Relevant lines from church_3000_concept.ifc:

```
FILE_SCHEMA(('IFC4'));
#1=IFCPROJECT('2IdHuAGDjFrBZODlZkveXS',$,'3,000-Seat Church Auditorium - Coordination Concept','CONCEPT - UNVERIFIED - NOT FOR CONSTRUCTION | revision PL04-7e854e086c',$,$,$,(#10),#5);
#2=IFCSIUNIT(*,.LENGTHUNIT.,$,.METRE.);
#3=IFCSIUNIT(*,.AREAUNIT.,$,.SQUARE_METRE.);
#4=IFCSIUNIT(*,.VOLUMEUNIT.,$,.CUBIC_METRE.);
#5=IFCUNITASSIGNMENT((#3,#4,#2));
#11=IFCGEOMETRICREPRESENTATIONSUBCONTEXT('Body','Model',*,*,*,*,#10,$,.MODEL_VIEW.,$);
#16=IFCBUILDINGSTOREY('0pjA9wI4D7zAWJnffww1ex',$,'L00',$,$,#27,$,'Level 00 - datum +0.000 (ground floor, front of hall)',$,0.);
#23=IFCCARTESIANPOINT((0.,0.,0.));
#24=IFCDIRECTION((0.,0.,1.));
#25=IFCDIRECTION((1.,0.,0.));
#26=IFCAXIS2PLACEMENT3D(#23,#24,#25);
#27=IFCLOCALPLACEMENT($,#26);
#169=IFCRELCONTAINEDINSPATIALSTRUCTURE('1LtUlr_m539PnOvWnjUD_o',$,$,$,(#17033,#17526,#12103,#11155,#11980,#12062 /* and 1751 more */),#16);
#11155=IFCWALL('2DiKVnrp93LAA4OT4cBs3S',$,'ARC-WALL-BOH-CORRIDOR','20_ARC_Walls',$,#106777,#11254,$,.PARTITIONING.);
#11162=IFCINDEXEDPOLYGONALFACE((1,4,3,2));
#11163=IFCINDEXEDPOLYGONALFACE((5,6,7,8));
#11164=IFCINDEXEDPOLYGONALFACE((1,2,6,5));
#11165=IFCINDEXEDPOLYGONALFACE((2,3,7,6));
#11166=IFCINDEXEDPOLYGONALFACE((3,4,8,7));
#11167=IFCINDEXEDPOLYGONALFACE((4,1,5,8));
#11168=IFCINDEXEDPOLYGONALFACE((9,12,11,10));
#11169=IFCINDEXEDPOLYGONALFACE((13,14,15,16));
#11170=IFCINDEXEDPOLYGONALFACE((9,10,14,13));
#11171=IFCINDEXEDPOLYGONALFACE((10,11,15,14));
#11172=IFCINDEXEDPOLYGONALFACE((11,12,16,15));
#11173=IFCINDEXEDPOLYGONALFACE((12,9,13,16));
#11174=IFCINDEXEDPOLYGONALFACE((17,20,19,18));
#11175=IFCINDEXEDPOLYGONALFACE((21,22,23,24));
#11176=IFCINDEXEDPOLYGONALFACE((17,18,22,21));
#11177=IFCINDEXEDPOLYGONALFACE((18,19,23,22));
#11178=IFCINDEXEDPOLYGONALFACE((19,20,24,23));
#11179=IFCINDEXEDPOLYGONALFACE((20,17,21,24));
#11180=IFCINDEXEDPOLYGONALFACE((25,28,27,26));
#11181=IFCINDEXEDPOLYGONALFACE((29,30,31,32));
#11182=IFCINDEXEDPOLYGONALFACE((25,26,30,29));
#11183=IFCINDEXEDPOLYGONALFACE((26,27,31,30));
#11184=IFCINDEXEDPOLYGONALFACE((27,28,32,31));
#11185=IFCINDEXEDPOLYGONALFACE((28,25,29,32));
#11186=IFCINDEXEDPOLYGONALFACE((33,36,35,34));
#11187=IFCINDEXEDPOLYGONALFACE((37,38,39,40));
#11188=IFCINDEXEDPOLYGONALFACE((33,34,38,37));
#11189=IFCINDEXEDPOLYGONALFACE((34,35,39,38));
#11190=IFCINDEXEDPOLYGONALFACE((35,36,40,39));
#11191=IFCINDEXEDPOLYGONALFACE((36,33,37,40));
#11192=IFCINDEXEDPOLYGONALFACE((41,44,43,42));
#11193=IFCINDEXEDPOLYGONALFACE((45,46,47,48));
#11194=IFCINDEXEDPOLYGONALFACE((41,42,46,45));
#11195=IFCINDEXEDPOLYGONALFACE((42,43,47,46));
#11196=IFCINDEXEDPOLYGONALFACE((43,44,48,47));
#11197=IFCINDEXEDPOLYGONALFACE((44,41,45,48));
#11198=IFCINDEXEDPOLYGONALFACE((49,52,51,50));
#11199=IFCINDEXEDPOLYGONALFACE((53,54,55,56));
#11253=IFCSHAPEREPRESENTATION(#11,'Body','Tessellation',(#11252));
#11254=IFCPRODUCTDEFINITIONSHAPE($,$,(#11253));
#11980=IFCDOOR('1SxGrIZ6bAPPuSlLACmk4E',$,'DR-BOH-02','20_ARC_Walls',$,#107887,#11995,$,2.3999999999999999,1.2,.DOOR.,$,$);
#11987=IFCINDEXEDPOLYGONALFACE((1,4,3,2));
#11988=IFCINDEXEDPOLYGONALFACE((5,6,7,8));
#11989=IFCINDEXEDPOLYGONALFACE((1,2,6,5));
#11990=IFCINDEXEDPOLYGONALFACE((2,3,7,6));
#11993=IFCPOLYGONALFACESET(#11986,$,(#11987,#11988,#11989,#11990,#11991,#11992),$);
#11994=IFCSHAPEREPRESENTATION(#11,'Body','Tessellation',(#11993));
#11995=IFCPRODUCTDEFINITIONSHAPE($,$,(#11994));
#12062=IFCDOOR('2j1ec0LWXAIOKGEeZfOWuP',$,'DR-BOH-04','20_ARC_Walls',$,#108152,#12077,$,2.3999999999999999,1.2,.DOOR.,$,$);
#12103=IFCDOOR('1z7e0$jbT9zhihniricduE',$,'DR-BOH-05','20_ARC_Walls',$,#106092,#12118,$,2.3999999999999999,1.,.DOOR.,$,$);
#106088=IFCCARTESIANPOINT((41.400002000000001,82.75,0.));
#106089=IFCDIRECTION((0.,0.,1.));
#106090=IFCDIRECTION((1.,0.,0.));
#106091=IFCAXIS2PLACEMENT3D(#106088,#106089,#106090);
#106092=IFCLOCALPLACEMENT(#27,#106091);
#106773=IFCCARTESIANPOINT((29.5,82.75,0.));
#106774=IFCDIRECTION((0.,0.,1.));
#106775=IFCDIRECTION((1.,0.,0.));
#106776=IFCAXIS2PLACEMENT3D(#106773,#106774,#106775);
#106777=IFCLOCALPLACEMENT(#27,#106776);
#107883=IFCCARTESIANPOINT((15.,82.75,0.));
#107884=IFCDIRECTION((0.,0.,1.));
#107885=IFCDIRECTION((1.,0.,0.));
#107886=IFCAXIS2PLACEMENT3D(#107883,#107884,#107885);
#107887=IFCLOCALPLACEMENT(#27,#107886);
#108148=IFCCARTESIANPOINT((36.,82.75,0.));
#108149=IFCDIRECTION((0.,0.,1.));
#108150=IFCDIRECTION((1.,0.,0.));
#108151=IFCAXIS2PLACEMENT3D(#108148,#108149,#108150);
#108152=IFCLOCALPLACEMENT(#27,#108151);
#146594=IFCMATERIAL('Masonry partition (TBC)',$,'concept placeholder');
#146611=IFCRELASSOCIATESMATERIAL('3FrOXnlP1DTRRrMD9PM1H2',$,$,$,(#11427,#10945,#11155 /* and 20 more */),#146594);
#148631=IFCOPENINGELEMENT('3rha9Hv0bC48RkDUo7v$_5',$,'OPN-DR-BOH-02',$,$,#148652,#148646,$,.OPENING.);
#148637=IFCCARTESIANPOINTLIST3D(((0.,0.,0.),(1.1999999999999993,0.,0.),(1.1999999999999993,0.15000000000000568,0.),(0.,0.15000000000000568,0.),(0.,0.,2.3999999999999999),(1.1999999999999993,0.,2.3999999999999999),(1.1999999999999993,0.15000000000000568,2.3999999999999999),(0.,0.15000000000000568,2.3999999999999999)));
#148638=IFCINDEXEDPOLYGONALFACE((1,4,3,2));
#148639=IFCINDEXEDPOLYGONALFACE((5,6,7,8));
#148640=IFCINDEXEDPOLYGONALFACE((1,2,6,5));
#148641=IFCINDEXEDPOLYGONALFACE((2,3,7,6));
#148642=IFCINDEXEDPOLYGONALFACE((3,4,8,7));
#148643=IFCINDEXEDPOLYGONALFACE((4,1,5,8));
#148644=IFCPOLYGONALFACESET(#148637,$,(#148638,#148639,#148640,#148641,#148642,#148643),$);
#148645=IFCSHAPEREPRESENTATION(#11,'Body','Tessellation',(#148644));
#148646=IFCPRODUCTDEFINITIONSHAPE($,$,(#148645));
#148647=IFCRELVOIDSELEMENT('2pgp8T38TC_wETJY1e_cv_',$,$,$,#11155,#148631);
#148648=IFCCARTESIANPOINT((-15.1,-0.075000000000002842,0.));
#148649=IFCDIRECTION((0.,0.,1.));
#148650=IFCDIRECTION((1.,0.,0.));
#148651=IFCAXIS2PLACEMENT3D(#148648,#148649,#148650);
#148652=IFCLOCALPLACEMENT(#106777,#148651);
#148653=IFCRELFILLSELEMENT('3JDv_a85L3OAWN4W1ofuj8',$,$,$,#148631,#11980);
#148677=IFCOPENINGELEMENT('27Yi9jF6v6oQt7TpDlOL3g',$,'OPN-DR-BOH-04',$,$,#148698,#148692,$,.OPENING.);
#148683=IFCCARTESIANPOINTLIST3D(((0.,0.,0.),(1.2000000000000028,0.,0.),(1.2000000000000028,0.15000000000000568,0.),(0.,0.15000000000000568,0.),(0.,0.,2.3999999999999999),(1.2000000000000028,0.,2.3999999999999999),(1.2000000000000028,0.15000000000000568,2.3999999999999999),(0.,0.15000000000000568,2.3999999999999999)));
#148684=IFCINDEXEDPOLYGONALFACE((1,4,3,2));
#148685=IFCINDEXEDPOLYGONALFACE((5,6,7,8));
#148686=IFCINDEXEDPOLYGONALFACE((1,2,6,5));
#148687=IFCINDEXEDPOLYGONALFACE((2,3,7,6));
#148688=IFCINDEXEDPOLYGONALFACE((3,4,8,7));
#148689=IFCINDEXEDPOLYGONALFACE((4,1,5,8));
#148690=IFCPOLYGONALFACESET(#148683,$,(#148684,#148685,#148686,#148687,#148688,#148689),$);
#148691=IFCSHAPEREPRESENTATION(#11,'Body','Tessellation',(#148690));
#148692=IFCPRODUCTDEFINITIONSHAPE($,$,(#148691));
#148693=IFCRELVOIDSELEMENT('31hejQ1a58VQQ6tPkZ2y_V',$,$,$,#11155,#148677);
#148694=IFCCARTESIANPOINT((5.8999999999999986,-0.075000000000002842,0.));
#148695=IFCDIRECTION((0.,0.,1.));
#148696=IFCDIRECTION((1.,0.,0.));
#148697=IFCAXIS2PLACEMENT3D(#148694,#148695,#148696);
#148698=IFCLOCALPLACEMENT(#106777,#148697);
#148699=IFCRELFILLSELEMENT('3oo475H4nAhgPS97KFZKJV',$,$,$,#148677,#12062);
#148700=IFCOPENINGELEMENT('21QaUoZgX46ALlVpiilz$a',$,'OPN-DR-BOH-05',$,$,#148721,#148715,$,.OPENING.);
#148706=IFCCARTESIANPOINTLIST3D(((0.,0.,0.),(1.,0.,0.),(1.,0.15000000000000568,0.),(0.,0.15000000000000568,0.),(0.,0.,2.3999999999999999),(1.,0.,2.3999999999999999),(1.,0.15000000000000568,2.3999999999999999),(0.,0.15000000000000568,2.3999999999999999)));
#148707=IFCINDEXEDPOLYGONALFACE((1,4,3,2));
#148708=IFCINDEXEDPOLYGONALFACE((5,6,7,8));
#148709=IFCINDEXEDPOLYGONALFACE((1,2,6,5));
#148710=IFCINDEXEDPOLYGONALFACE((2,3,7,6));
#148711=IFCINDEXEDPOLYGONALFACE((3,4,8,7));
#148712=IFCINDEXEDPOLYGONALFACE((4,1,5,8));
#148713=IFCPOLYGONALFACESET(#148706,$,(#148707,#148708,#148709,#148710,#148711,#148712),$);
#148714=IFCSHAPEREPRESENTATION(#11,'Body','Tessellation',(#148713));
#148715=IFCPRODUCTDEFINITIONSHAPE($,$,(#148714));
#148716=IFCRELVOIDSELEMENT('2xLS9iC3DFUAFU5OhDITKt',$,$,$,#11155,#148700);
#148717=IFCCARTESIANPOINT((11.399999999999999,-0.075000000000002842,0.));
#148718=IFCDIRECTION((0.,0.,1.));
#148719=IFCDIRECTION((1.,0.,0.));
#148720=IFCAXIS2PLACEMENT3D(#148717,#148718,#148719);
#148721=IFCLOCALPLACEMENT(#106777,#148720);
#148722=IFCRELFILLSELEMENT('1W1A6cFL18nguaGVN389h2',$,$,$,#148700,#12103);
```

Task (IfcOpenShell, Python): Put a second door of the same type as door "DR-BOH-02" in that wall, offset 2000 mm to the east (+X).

```python
import ifcopenshell
import ifcopenshell.api.feature
import ifcopenshell.api.geometry
import ifcopenshell.api.root
import ifcopenshell.geom
import ifcopenshell.util.element
import ifcopenshell.util.placement
import ifcopenshell.util.shape
import ifcopenshell.util.unit

model = ifcopenshell.open("church_3000_concept.ifc")
unit_scale = ifcopenshell.util.unit.calculate_unit_scale(model)
settings = ifcopenshell.geom.settings()


def volume(element):
    """Net volume in cubic metres, openings subtracted."""
    shape = ifcopenshell.geom.create_shape(settings, element)
    return ifcopenshell.util.shape.get_volume(shape.geometry)


door = model.by_guid("1SxGrIZ6bAPPuSlLACmk4E")
opening = door.FillsVoids[0].RelatingOpeningElement
wall = opening.VoidsElements[0].RelatingBuildingElement
before = volume(wall)
shift = ifcopenshell.util.placement.get_local_placement(wall.ObjectPlacement)[:3, 0] * 2 / unit_scale

# copy_class copies the void relationship, type, container and properties, but no geometry.
new_opening = ifcopenshell.api.root.copy_class(model, product=opening)
new_opening.Representation = ifcopenshell.util.element.copy_deep(
    model, opening.Representation, exclude=["IfcGeometricRepresentationContext", "IfcRepresentationMap"]
)
new_door = ifcopenshell.api.root.copy_class(model, product=door)
new_door.Representation = ifcopenshell.util.element.copy_deep(
    model, door.Representation, exclude=["IfcGeometricRepresentationContext", "IfcRepresentationMap"]
)
ifcopenshell.api.feature.add_filling(model, opening=new_opening, element=new_door)

for old, new in ((opening, new_opening), (door, new_door)):
    matrix = ifcopenshell.util.placement.get_local_placement(old.ObjectPlacement)
    matrix[:3, 3] += shift
    ifcopenshell.api.geometry.edit_object_placement(model, product=new, matrix=matrix, is_si=False)

after = volume(wall)

print(f"wall volume {before:.3f} -> {after:.3f} m3")

model.write("church_3000_concept-out.ifc")
```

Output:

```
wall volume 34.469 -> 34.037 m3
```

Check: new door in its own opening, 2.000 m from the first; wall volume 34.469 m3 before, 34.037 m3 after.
